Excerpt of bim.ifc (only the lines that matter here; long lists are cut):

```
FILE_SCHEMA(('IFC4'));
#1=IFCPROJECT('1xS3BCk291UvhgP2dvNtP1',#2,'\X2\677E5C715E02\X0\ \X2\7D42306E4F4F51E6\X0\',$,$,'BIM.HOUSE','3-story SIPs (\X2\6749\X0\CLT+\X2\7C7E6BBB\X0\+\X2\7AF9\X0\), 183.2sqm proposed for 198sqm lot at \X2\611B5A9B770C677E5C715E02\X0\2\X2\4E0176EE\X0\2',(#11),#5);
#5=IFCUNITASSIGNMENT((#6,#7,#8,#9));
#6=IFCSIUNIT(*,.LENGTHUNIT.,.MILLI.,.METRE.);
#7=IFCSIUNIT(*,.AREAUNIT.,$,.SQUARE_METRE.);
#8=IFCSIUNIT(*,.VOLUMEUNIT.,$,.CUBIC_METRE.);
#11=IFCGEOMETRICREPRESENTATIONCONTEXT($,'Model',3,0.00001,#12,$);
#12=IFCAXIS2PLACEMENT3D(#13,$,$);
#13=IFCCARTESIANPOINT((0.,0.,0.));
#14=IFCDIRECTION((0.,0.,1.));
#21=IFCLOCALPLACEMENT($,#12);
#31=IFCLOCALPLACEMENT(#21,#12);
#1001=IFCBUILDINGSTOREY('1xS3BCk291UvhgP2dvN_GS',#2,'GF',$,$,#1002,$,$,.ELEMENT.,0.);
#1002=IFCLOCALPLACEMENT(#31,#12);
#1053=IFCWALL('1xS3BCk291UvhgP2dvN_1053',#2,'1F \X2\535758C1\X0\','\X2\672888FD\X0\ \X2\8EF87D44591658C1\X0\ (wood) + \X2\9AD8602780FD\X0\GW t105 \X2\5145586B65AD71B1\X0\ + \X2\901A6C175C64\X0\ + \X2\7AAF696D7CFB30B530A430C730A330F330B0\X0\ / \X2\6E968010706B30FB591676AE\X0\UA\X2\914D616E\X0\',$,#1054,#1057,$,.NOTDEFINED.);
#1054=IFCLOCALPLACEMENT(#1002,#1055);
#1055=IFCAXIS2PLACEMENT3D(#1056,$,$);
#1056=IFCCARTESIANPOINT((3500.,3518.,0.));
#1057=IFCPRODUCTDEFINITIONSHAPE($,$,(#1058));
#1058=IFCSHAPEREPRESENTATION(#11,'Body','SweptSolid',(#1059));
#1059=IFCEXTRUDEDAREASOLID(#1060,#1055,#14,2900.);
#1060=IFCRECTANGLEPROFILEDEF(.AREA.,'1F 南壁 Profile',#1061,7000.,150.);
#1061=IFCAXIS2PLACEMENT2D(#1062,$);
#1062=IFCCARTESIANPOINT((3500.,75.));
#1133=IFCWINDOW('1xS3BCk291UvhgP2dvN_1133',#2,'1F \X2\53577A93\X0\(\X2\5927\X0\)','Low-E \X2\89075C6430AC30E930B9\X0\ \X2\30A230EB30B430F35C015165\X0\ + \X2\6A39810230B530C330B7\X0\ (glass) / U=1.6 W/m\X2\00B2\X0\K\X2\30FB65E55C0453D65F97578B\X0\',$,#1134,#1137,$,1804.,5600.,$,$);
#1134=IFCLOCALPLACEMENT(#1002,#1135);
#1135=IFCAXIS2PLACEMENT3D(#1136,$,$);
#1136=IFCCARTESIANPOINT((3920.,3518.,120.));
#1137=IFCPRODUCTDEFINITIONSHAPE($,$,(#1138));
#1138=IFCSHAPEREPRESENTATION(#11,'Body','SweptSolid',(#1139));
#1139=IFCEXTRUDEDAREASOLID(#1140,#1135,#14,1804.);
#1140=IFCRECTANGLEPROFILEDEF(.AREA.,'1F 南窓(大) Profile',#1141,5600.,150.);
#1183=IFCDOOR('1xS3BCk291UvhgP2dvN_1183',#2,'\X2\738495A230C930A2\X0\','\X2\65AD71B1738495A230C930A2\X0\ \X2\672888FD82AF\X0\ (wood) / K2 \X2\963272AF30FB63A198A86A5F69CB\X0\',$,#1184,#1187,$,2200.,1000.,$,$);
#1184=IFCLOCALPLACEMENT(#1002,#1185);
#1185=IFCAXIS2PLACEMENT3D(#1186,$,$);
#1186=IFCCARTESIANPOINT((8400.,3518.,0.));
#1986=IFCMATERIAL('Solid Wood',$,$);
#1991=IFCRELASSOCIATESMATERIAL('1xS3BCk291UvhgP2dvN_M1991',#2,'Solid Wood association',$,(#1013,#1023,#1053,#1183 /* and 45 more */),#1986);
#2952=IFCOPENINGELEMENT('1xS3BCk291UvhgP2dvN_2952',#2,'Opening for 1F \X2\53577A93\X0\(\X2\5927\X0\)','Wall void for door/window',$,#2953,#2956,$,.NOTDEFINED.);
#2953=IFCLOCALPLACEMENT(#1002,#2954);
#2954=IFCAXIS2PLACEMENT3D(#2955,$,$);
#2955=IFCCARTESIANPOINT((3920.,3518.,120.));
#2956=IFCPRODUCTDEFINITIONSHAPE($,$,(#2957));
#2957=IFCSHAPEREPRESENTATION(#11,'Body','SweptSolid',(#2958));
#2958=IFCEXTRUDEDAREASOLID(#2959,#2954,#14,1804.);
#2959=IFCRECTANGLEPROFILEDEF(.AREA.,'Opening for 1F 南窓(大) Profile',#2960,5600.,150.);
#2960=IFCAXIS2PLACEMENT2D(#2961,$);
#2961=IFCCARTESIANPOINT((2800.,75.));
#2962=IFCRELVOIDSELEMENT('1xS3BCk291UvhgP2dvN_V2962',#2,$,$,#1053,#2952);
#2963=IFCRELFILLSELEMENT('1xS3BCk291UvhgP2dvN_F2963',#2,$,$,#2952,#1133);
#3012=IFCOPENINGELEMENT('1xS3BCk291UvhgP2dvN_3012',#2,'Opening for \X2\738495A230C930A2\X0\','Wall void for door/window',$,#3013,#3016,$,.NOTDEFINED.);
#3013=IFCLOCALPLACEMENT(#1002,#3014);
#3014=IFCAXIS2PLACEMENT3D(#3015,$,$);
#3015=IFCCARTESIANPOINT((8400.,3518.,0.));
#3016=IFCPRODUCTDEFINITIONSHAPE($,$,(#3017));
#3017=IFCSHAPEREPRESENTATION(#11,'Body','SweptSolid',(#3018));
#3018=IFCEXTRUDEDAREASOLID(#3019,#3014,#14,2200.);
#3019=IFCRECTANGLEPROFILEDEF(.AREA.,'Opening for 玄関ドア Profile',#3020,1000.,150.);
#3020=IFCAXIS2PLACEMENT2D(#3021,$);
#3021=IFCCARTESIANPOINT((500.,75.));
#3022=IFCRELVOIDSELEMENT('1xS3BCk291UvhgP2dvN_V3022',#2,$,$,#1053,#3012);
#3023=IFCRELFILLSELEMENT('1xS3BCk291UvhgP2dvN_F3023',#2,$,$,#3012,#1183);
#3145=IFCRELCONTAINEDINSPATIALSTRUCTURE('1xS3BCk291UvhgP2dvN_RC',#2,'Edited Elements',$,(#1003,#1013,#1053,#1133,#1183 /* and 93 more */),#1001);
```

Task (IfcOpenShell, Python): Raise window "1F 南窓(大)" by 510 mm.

```python
import numpy as np
import ifcopenshell
import ifcopenshell.api.geometry
import ifcopenshell.util.placement
import ifcopenshell.util.unit

model = ifcopenshell.open("bim.ifc")
unit_scale = ifcopenshell.util.unit.calculate_unit_scale(model)

window = model.by_id(1133)
opening = window.FillsVoids[0].RelatingOpeningElement
dz = 0.51 / unit_scale

shift = np.array([0.0, 0.0, dz])
# The window is not placed relative to its opening, so move both.
for product in (opening, window):
    matrix = ifcopenshell.util.placement.get_local_placement(product.ObjectPlacement)
    matrix[:3, 3] += shift
    ifcopenshell.api.geometry.edit_object_placement(model, product=product, matrix=matrix, is_si=False)

print(f"moved by {dz * unit_scale:+.3f} m")

model.write("bim-out.ifc")
```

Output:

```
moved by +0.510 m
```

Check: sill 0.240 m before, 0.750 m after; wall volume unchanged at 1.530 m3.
